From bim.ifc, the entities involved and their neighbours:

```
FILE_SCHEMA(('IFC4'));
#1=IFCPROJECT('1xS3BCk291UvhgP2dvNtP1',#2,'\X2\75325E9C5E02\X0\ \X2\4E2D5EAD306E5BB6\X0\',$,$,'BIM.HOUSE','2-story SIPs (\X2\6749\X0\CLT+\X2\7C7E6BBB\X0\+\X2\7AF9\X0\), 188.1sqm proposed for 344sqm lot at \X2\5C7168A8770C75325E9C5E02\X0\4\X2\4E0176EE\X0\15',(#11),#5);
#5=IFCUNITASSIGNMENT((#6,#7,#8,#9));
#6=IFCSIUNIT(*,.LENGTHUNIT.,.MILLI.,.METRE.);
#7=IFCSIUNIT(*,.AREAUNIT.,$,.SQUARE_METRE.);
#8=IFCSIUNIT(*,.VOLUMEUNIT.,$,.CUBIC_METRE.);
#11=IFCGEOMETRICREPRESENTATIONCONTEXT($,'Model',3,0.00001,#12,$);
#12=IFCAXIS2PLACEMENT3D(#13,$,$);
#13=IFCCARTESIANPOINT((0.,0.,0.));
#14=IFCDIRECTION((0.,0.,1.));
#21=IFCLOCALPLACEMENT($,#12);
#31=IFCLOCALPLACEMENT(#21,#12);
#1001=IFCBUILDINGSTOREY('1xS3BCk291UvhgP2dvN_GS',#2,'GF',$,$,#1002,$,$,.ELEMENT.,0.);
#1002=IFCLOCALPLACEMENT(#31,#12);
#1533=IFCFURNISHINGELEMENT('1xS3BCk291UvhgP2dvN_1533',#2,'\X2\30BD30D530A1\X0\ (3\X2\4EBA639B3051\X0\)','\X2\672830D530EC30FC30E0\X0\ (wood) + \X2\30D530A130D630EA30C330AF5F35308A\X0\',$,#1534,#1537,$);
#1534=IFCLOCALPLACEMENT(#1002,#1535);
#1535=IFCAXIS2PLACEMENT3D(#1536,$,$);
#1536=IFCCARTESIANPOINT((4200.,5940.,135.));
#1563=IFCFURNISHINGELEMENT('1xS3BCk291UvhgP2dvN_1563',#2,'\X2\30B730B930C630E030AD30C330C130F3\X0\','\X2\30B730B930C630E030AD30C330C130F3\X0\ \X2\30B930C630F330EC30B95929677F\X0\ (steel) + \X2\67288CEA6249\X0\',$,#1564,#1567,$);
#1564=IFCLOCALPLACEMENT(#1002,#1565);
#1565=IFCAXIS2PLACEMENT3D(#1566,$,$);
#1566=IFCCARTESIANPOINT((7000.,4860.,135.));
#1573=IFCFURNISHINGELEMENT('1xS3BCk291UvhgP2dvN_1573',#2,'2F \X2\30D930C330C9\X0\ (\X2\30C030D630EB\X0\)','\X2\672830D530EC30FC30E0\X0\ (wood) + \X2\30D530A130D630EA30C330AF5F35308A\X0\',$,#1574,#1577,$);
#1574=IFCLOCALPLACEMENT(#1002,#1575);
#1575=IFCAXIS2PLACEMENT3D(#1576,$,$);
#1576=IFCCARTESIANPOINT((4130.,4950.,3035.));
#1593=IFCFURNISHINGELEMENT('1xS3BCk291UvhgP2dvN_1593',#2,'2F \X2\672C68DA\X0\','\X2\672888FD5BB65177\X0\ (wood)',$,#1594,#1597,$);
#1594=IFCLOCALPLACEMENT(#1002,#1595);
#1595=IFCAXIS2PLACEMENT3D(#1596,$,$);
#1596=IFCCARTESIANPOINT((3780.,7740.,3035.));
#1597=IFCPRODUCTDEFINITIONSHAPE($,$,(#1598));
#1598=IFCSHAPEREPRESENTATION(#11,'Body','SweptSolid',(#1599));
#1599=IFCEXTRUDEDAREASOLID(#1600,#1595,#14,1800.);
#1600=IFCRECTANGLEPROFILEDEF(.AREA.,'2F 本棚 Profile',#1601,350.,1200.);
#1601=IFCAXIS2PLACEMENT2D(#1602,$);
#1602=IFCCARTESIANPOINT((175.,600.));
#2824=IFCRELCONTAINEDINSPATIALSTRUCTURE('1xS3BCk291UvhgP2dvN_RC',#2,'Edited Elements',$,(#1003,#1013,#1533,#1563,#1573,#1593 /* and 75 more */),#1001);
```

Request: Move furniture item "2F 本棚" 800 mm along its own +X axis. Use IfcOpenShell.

```python
import ifcopenshell
import ifcopenshell.api.geometry
import ifcopenshell.util.placement
import ifcopenshell.util.unit

model = ifcopenshell.open("bim.ifc")
unit_scale = ifcopenshell.util.unit.calculate_unit_scale(model)

item = model.by_guid("1xS3BCk291UvhgP2dvN_1593")
matrix = ifcopenshell.util.placement.get_local_placement(item.ObjectPlacement)
matrix[:3, 3] += matrix[:3, 0] * 0.8 / unit_scale
ifcopenshell.api.geometry.edit_object_placement(model, product=item, matrix=matrix, is_si=False)

print(ifcopenshell.util.placement.get_local_placement(item.ObjectPlacement).round(3) + 0.0)

model.write("bim_rev.ifc")
```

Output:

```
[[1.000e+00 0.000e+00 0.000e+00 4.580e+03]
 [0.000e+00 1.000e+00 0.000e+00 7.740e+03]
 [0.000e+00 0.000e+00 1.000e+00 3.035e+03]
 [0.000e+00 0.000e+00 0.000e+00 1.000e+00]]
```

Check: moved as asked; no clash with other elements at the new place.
